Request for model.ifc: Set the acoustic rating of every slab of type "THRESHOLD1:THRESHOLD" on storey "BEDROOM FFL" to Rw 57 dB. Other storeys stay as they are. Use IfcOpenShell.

First a look at what the model holds.

```python
import ifcopenshell
import ifcopenshell.util.element

model = ifcopenshell.open("model.ifc")
print(model.schema)
storey = next(s for s in model.by_type("IfcBuildingStorey") if s.Name == "BEDROOM FFL")
slabs = [e for e in ifcopenshell.util.element.get_decomposition(storey) if e.is_a("IfcSlab")]
seen = {}
for e in slabs:
    element_type = ifcopenshell.util.element.get_type(e)
    key = (element_type.Name if element_type != e and element_type else None, ifcopenshell.util.element.get_pset(e, "Pset_SlabCommon", "AcousticRating"))
    seen[key] = seen.get(key, 0) + 1
for (name, value), count in sorted(seen.items(), key=str):
    print(count, "x", name, "|", value)
```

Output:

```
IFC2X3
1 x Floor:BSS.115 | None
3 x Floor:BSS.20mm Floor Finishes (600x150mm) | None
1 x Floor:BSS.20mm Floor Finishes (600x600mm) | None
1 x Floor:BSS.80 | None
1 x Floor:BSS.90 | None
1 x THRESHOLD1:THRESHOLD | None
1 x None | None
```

```python
import ifcopenshell
import ifcopenshell.api.pset
import ifcopenshell.util.element

model = ifcopenshell.open("model.ifc")

storey = next(s for s in model.by_type("IfcBuildingStorey") if s.Name == "BEDROOM FFL")
slabs = [e for e in ifcopenshell.util.element.get_decomposition(storey) if e.is_a("IfcSlab")]

count = 0
for e in slabs:
    element_type = ifcopenshell.util.element.get_type(e)
    if element_type in (None, e) or element_type.Name != "THRESHOLD1:THRESHOLD":
        continue
    # add_pset returns the element's existing set when there is one.
    pset = ifcopenshell.api.pset.add_pset(model, product=e, name="Pset_SlabCommon")
    ifcopenshell.api.pset.edit_pset(model, pset=pset, properties={"AcousticRating": "Rw 57 dB"})
    count += 1

print(count, "slabs updated")

model.write("model-out.ifc")
```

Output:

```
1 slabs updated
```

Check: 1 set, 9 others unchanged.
